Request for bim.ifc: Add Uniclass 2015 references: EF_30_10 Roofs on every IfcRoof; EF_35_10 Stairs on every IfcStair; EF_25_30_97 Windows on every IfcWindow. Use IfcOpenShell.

First a look at what the model holds.

```python
import ifcopenshell

model = ifcopenshell.open("bim.ifc")
print(model.schema)
print("classifications:", [c.Name for c in model.by_type("IfcClassification")])
for ifc_class in ("IfcDoor", "IfcRoof", "IfcStair", "IfcWall", "IfcWindow"):
    print(ifc_class, len(model.by_type(ifc_class)))
```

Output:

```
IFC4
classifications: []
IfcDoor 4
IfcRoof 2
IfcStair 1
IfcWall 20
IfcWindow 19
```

```python
import ifcopenshell
import ifcopenshell.api.classification

model = ifcopenshell.open("bim.ifc")

system = ifcopenshell.api.classification.add_classification(model, classification="Uniclass 2015")

codes = {
    "IfcRoof": ("EF_30_10", "Roofs"),
    "IfcStair": ("EF_35_10", "Stairs"),
    "IfcWindow": ("EF_25_30_97", "Windows"),
}
for ifc_class, (code, name) in codes.items():
    products = model.by_type(ifc_class)
    ifcopenshell.api.classification.add_reference(
        model, products=products, classification=system, identification=code, name=name
    )
    print(code, len(products))

model.write("bim_rev.ifc")
```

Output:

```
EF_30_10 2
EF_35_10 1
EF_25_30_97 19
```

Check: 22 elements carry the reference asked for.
